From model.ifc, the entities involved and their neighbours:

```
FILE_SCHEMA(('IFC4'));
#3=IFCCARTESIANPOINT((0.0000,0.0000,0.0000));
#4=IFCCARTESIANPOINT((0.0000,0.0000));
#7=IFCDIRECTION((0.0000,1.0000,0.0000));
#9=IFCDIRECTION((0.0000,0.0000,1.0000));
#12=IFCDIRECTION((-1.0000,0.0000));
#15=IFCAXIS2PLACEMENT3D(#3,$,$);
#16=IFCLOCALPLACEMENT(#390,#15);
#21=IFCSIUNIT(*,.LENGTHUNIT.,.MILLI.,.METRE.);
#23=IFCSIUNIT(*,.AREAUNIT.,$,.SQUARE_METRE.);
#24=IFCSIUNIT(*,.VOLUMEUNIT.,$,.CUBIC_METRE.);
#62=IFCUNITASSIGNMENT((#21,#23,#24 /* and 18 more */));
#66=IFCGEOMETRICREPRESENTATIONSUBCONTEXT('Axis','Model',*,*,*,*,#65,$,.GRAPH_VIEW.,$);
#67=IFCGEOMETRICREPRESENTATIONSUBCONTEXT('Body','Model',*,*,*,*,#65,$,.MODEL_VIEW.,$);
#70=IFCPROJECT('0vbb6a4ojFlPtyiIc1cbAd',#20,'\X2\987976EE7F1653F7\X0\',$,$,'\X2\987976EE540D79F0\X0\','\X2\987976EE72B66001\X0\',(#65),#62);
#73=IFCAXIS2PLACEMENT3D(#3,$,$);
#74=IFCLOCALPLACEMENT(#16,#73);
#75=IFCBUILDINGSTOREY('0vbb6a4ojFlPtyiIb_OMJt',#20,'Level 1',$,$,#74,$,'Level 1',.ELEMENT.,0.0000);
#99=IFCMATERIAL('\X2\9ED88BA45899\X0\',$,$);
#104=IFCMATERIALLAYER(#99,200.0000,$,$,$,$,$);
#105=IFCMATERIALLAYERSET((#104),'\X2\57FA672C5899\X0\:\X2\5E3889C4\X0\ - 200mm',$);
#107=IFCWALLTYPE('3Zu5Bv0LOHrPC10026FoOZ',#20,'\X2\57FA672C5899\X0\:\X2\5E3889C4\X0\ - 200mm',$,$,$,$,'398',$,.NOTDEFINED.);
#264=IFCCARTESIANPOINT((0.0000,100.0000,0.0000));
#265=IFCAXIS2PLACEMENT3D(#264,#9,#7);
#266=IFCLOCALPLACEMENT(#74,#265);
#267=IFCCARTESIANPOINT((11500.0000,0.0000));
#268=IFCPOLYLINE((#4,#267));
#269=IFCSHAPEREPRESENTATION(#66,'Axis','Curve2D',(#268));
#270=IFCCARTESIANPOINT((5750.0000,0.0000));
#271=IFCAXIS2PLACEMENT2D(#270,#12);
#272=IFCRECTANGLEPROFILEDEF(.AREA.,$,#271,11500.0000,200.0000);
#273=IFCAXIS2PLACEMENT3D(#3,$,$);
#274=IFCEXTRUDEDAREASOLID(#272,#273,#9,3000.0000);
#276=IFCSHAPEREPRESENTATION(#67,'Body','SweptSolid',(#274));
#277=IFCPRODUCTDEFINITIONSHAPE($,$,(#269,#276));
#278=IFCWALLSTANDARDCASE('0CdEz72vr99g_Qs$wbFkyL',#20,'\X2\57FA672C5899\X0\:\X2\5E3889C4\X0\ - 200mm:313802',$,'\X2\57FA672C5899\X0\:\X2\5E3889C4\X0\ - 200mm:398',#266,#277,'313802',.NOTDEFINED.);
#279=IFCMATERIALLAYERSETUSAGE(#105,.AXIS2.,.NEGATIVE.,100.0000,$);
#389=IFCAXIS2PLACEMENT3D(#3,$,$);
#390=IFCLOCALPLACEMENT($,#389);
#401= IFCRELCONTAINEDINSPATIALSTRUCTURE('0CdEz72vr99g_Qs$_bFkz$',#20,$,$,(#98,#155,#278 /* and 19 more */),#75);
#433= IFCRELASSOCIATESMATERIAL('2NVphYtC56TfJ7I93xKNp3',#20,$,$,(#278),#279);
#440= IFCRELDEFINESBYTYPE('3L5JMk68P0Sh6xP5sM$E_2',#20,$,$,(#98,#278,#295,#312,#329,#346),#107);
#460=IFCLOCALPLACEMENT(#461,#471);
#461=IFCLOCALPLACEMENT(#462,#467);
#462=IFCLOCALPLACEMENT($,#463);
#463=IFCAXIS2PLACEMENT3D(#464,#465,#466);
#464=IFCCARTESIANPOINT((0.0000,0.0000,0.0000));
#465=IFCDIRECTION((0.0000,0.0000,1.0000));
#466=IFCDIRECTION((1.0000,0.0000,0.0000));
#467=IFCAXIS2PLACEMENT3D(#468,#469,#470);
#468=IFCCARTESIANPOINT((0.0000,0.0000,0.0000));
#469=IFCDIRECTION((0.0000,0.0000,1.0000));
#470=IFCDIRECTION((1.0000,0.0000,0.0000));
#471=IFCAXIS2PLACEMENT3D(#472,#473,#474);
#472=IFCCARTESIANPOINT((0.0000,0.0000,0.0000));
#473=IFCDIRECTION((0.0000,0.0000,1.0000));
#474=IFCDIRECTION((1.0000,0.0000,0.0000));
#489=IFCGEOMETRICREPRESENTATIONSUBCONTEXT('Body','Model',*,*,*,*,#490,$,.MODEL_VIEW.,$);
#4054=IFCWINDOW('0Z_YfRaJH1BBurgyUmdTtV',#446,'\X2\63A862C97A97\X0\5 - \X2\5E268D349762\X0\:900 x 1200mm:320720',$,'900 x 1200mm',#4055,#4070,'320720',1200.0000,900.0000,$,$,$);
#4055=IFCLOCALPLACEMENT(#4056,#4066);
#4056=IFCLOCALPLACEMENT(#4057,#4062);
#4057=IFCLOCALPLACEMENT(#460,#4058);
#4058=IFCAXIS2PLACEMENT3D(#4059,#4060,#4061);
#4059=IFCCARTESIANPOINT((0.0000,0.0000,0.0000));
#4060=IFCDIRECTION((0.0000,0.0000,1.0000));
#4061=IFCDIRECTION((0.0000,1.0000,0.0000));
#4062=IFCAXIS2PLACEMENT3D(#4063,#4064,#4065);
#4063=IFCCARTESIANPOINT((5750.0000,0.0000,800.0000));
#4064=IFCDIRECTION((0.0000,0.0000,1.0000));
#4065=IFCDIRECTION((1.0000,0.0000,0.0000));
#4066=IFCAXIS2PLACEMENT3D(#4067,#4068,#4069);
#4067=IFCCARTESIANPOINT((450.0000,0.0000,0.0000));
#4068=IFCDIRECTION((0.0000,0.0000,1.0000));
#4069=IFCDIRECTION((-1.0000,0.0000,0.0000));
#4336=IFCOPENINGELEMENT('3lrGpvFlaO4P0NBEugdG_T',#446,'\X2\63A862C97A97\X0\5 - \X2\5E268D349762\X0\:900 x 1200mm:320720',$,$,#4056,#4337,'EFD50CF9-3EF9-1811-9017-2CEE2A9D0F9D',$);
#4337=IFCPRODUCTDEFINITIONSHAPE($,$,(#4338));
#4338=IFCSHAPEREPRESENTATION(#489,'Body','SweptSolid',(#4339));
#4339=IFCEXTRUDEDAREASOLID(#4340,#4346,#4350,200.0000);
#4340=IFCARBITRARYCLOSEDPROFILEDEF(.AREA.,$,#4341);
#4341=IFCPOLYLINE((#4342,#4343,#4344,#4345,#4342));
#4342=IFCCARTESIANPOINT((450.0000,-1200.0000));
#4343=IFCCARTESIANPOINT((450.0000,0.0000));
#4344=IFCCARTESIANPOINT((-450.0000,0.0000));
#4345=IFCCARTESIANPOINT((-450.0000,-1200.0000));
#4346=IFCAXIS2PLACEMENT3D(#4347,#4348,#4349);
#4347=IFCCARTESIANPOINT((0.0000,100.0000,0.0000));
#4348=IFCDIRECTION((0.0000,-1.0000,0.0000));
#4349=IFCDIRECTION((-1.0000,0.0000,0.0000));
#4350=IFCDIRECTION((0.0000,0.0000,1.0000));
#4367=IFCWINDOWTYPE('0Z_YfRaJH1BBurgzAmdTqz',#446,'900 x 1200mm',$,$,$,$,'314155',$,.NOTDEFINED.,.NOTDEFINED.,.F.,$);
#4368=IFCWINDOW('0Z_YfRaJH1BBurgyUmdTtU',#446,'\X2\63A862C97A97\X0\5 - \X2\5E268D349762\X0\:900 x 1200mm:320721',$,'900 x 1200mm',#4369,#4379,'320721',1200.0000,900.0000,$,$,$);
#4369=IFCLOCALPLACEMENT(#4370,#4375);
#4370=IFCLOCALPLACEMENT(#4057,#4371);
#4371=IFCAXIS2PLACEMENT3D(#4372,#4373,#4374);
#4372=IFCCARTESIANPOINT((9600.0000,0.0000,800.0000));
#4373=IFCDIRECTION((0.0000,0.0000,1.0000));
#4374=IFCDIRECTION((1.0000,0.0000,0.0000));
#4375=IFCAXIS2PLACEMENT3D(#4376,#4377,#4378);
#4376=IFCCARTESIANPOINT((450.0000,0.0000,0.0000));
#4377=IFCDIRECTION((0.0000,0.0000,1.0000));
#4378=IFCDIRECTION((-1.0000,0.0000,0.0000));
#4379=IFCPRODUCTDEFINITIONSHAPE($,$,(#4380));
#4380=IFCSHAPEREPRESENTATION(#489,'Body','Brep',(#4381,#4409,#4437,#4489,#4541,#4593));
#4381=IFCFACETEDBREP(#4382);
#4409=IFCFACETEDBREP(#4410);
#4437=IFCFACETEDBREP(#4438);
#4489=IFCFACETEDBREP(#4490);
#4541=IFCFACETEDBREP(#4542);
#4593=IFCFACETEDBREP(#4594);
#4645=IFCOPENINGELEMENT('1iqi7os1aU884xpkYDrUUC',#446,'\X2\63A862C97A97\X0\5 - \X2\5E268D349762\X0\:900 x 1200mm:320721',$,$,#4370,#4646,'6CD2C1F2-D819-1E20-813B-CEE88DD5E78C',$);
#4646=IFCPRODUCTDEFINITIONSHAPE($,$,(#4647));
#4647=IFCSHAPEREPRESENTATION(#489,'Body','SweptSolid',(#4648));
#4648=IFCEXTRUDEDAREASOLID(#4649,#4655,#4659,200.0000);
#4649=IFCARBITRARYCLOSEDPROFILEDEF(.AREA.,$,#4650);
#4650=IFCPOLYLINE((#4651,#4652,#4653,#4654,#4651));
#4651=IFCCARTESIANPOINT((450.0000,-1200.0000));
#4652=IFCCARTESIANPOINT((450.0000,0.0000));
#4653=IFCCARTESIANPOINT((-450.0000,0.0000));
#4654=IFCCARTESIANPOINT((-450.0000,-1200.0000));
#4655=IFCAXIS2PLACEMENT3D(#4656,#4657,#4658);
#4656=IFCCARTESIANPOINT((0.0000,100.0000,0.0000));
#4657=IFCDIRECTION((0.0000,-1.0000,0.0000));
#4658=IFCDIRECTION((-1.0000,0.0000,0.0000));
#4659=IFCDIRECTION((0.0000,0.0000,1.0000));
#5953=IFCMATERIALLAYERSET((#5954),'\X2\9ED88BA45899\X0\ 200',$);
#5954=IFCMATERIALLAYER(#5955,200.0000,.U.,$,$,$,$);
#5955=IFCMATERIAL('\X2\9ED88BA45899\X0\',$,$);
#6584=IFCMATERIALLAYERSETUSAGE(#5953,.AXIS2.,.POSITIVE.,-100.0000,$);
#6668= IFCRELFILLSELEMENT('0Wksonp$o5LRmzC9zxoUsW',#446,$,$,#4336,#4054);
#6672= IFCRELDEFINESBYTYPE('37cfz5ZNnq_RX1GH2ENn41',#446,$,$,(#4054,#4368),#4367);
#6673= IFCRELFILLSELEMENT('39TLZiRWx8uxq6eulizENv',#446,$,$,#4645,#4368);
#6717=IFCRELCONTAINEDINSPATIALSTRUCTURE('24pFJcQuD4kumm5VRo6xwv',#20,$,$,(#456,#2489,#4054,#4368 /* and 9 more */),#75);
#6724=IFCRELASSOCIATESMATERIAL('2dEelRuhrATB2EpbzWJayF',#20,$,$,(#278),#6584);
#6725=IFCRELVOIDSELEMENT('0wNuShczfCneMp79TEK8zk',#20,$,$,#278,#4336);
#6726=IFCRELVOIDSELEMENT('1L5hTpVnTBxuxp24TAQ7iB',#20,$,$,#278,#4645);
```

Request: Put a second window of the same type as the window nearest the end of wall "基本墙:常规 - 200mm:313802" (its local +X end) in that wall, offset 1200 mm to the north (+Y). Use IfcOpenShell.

```python
import ifcopenshell
import ifcopenshell.api.feature
import ifcopenshell.api.geometry
import ifcopenshell.api.root
import ifcopenshell.geom
import ifcopenshell.util.element
import ifcopenshell.util.placement
import ifcopenshell.util.shape
import ifcopenshell.util.unit

model = ifcopenshell.open("model.ifc")
unit_scale = ifcopenshell.util.unit.calculate_unit_scale(model)
settings = ifcopenshell.geom.settings()


def volume(element):
    """Net volume in cubic metres, openings subtracted."""
    shape = ifcopenshell.geom.create_shape(settings, element)
    return ifcopenshell.util.shape.get_volume(shape.geometry)


def reuse_history(source, copy):
    """copy_class also copies each property set's owner history, people and application; keep the originals."""
    for rel in copy.IsDefinedBy:
        if rel.is_a("IfcRelDefinesByProperties") and (history := rel.RelatingPropertyDefinition.OwnerHistory):
            rel.RelatingPropertyDefinition.OwnerHistory = source.OwnerHistory
            ifcopenshell.util.element.remove_deep2(model, history)


window = model.by_guid("0Z_YfRaJH1BBurgyUmdTtU")
opening = window.FillsVoids[0].RelatingOpeningElement
wall = opening.VoidsElements[0].RelatingBuildingElement
before = volume(wall)
shift = ifcopenshell.util.placement.get_local_placement(wall.ObjectPlacement)[:3, 0] * 1.2 / unit_scale

# copy_class copies the void relationship, type, container and properties, but no geometry.
new_opening = ifcopenshell.api.root.copy_class(model, product=opening)
new_opening.Representation = ifcopenshell.util.element.copy_deep(
    model, opening.Representation, exclude=["IfcGeometricRepresentationContext", "IfcRepresentationMap"]
)
new_opening.Name = "推拉窗5 - 带贴面:900 x 1200mm"
new_opening.Tag = None
new_window = ifcopenshell.api.root.copy_class(model, product=window)
new_window.Representation = ifcopenshell.util.element.copy_deep(
    model, window.Representation, exclude=["IfcGeometricRepresentationContext", "IfcRepresentationMap"]
)
new_window.Name = "推拉窗5 - 带贴面:900 x 1200mm"
new_window.Tag = None
reuse_history(window, new_window)
ifcopenshell.api.feature.add_filling(model, opening=new_opening, element=new_window)

for old, new in ((opening, new_opening), (window, new_window)):
    matrix = ifcopenshell.util.placement.get_local_placement(old.ObjectPlacement)
    matrix[:3, 3] += shift
    ifcopenshell.api.geometry.edit_object_placement(model, product=new, matrix=matrix, is_si=False)

after = volume(wall)

print(f"wall volume {before:.3f} -> {after:.3f} m3")

model.write("model-out.ifc")
```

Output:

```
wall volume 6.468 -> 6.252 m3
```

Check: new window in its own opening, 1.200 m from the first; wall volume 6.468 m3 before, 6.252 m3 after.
